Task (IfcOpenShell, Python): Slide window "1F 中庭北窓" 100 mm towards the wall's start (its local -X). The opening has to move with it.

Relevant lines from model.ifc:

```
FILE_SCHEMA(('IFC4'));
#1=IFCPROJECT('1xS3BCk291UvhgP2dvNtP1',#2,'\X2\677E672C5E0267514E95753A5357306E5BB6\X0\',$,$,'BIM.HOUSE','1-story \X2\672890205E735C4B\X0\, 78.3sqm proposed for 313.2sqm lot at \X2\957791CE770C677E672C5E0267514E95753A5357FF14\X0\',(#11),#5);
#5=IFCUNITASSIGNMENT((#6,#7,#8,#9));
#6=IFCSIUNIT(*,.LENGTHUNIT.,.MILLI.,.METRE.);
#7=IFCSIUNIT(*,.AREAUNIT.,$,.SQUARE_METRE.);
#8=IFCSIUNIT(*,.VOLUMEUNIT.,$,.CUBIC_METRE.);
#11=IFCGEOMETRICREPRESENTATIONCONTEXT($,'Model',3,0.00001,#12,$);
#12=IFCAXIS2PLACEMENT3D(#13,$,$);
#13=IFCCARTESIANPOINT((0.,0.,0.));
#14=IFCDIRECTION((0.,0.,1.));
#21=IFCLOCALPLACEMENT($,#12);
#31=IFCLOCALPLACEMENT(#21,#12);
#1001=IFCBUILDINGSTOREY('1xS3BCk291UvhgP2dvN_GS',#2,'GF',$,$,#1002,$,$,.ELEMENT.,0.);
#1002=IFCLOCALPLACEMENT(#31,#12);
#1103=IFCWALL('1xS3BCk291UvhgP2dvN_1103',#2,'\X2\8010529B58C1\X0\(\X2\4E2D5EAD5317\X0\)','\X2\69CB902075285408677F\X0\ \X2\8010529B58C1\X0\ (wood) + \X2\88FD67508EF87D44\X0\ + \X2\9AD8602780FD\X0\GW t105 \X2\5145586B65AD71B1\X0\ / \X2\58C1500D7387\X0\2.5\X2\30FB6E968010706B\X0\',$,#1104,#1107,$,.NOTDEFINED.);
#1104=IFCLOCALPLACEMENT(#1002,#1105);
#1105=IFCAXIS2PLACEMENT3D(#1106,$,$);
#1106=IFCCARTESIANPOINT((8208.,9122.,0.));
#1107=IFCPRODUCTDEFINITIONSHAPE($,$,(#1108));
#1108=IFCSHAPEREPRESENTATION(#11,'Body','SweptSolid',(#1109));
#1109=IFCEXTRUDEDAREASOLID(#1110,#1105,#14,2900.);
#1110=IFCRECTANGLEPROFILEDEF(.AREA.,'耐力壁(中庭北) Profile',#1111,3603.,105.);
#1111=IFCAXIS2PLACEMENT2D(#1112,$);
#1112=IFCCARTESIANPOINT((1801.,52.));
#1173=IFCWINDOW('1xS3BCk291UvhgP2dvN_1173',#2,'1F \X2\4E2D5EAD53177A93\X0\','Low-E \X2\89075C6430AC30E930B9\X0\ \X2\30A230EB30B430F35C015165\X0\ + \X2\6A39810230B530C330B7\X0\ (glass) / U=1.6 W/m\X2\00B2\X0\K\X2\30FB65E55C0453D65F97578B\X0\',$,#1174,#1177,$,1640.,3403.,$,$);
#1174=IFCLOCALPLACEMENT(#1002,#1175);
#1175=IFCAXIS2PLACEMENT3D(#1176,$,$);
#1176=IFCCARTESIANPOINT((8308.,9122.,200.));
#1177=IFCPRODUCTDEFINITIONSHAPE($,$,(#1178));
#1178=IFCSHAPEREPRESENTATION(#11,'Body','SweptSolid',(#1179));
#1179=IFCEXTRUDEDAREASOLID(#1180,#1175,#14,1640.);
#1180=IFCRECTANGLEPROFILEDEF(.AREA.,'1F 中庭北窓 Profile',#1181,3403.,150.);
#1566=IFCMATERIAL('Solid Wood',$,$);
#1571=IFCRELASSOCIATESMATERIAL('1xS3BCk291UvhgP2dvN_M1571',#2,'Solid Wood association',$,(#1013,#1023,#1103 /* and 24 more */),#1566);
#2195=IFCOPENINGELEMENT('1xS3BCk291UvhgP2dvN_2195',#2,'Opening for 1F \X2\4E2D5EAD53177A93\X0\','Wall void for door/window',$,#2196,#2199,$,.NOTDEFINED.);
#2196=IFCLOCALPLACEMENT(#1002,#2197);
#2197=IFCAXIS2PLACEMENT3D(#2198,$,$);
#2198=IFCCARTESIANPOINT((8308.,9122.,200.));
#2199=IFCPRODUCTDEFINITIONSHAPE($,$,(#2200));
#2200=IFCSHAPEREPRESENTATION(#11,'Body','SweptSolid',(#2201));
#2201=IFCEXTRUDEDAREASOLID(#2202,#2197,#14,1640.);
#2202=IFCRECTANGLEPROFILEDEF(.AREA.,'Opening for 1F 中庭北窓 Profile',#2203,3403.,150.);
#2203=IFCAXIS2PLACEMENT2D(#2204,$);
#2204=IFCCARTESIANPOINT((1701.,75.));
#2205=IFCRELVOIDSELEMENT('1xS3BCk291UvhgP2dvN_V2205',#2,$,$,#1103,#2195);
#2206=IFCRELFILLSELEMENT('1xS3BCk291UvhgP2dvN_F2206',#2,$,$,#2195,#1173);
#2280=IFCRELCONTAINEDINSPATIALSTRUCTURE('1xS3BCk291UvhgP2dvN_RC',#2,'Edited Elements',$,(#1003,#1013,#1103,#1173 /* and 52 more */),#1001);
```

```python
import ifcopenshell
import ifcopenshell.api.geometry
import ifcopenshell.util.placement
import ifcopenshell.util.unit

model = ifcopenshell.open("model.ifc")
unit_scale = ifcopenshell.util.unit.calculate_unit_scale(model)

window = model.by_guid("1xS3BCk291UvhgP2dvN_1173")
opening = window.FillsVoids[0].RelatingOpeningElement
wall = opening.VoidsElements[0].RelatingBuildingElement

wall_matrix = ifcopenshell.util.placement.get_local_placement(wall.ObjectPlacement)
shift = wall_matrix[:3, 0] * -0.1 / unit_scale
before = ifcopenshell.util.placement.get_local_placement(window.ObjectPlacement)[:3, 3].copy()

# The window is not placed relative to its opening, so move both.
for product in (opening, window):
    matrix = ifcopenshell.util.placement.get_local_placement(product.ObjectPlacement)
    matrix[:3, 3] += shift
    ifcopenshell.api.geometry.edit_object_placement(model, product=product, matrix=matrix, is_si=False)

after = ifcopenshell.util.placement.get_local_placement(window.ObjectPlacement)[:3, 3]
print("window moved by", (after - before).round(3) + 0.0)

model.write("model_edited.ifc")
```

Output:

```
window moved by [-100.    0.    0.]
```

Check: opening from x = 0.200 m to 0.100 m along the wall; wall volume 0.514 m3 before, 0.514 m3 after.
